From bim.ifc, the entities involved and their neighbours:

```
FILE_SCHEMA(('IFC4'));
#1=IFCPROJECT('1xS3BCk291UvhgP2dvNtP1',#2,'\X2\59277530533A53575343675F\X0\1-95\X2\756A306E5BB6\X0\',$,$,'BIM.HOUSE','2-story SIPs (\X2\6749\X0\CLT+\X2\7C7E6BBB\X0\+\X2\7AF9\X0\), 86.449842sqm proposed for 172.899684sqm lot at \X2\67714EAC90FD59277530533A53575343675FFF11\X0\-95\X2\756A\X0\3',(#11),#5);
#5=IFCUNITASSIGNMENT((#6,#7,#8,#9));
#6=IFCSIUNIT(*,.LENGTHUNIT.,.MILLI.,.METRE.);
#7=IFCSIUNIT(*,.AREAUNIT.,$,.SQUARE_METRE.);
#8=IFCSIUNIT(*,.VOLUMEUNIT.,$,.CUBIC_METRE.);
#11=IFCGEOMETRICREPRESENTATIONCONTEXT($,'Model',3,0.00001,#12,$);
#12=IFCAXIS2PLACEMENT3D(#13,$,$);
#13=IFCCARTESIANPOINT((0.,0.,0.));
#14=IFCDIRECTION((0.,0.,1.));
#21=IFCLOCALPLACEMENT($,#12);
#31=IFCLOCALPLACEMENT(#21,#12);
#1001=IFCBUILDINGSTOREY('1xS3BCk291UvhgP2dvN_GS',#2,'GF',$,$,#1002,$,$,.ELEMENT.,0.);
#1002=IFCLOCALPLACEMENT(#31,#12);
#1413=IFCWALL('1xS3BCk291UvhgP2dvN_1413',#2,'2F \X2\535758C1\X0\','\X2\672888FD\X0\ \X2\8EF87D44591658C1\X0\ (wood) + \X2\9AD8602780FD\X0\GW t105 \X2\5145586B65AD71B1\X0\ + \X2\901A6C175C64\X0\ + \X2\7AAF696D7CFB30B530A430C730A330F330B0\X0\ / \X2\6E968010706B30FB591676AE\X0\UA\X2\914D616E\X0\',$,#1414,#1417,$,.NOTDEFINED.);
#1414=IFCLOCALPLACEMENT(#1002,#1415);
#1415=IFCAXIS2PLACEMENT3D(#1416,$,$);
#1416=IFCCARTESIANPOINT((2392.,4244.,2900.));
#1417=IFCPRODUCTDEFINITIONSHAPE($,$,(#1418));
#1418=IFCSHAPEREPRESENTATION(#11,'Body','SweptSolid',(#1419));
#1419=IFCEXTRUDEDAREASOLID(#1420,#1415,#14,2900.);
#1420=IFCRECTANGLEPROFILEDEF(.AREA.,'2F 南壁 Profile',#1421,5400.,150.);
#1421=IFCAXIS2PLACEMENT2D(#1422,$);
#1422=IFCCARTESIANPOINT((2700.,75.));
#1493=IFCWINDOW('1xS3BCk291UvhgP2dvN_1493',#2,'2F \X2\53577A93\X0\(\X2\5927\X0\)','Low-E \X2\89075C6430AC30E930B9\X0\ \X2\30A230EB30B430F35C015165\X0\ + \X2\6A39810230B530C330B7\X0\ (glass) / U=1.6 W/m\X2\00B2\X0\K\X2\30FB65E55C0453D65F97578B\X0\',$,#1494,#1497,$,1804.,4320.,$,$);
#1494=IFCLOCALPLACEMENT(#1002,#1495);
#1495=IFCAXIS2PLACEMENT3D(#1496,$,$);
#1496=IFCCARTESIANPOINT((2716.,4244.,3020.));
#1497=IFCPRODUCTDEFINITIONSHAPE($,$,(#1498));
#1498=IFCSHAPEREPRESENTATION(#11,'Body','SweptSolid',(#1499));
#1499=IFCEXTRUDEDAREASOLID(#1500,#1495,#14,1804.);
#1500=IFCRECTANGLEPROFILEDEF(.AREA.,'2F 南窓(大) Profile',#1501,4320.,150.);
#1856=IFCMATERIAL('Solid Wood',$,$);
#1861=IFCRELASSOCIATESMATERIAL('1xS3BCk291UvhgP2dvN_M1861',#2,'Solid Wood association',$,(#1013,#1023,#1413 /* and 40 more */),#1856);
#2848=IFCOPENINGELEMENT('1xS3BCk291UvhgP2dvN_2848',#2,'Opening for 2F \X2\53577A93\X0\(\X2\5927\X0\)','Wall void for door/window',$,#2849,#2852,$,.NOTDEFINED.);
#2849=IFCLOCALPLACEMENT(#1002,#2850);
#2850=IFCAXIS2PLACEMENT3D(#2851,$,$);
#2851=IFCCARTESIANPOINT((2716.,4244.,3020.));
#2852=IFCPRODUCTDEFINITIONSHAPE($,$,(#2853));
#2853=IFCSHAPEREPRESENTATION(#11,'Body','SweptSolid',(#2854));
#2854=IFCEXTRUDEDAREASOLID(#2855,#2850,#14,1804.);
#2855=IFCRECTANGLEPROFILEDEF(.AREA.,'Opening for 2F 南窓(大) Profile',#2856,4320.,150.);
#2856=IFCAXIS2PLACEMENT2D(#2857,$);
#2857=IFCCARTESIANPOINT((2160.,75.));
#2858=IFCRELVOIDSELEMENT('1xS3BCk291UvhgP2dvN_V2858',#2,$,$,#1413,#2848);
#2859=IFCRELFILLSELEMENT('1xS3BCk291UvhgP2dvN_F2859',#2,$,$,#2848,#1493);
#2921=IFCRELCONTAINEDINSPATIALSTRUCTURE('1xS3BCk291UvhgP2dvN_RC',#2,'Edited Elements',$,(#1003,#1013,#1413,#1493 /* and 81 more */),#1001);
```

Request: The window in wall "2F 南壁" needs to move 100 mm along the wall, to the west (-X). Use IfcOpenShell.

```python
import ifcopenshell
import ifcopenshell.api.geometry
import ifcopenshell.util.placement
import ifcopenshell.util.unit

model = ifcopenshell.open("bim.ifc")
unit_scale = ifcopenshell.util.unit.calculate_unit_scale(model)

window = model.by_guid("1xS3BCk291UvhgP2dvN_1493")
opening = window.FillsVoids[0].RelatingOpeningElement
wall = opening.VoidsElements[0].RelatingBuildingElement

wall_matrix = ifcopenshell.util.placement.get_local_placement(wall.ObjectPlacement)
shift = wall_matrix[:3, 0] * -0.1 / unit_scale
before = ifcopenshell.util.placement.get_local_placement(window.ObjectPlacement)[:3, 3].copy()

# The window is not placed relative to its opening, so move both.
for product in (opening, window):
    matrix = ifcopenshell.util.placement.get_local_placement(product.ObjectPlacement)
    matrix[:3, 3] += shift
    ifcopenshell.api.geometry.edit_object_placement(model, product=product, matrix=matrix, is_si=False)

after = ifcopenshell.util.placement.get_local_placement(window.ObjectPlacement)[:3, 3]
print("window moved by", (after - before).round(3) + 0.0)

model.write("bim_rev.ifc")
```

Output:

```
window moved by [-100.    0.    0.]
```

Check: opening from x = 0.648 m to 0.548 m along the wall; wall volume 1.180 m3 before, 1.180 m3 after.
